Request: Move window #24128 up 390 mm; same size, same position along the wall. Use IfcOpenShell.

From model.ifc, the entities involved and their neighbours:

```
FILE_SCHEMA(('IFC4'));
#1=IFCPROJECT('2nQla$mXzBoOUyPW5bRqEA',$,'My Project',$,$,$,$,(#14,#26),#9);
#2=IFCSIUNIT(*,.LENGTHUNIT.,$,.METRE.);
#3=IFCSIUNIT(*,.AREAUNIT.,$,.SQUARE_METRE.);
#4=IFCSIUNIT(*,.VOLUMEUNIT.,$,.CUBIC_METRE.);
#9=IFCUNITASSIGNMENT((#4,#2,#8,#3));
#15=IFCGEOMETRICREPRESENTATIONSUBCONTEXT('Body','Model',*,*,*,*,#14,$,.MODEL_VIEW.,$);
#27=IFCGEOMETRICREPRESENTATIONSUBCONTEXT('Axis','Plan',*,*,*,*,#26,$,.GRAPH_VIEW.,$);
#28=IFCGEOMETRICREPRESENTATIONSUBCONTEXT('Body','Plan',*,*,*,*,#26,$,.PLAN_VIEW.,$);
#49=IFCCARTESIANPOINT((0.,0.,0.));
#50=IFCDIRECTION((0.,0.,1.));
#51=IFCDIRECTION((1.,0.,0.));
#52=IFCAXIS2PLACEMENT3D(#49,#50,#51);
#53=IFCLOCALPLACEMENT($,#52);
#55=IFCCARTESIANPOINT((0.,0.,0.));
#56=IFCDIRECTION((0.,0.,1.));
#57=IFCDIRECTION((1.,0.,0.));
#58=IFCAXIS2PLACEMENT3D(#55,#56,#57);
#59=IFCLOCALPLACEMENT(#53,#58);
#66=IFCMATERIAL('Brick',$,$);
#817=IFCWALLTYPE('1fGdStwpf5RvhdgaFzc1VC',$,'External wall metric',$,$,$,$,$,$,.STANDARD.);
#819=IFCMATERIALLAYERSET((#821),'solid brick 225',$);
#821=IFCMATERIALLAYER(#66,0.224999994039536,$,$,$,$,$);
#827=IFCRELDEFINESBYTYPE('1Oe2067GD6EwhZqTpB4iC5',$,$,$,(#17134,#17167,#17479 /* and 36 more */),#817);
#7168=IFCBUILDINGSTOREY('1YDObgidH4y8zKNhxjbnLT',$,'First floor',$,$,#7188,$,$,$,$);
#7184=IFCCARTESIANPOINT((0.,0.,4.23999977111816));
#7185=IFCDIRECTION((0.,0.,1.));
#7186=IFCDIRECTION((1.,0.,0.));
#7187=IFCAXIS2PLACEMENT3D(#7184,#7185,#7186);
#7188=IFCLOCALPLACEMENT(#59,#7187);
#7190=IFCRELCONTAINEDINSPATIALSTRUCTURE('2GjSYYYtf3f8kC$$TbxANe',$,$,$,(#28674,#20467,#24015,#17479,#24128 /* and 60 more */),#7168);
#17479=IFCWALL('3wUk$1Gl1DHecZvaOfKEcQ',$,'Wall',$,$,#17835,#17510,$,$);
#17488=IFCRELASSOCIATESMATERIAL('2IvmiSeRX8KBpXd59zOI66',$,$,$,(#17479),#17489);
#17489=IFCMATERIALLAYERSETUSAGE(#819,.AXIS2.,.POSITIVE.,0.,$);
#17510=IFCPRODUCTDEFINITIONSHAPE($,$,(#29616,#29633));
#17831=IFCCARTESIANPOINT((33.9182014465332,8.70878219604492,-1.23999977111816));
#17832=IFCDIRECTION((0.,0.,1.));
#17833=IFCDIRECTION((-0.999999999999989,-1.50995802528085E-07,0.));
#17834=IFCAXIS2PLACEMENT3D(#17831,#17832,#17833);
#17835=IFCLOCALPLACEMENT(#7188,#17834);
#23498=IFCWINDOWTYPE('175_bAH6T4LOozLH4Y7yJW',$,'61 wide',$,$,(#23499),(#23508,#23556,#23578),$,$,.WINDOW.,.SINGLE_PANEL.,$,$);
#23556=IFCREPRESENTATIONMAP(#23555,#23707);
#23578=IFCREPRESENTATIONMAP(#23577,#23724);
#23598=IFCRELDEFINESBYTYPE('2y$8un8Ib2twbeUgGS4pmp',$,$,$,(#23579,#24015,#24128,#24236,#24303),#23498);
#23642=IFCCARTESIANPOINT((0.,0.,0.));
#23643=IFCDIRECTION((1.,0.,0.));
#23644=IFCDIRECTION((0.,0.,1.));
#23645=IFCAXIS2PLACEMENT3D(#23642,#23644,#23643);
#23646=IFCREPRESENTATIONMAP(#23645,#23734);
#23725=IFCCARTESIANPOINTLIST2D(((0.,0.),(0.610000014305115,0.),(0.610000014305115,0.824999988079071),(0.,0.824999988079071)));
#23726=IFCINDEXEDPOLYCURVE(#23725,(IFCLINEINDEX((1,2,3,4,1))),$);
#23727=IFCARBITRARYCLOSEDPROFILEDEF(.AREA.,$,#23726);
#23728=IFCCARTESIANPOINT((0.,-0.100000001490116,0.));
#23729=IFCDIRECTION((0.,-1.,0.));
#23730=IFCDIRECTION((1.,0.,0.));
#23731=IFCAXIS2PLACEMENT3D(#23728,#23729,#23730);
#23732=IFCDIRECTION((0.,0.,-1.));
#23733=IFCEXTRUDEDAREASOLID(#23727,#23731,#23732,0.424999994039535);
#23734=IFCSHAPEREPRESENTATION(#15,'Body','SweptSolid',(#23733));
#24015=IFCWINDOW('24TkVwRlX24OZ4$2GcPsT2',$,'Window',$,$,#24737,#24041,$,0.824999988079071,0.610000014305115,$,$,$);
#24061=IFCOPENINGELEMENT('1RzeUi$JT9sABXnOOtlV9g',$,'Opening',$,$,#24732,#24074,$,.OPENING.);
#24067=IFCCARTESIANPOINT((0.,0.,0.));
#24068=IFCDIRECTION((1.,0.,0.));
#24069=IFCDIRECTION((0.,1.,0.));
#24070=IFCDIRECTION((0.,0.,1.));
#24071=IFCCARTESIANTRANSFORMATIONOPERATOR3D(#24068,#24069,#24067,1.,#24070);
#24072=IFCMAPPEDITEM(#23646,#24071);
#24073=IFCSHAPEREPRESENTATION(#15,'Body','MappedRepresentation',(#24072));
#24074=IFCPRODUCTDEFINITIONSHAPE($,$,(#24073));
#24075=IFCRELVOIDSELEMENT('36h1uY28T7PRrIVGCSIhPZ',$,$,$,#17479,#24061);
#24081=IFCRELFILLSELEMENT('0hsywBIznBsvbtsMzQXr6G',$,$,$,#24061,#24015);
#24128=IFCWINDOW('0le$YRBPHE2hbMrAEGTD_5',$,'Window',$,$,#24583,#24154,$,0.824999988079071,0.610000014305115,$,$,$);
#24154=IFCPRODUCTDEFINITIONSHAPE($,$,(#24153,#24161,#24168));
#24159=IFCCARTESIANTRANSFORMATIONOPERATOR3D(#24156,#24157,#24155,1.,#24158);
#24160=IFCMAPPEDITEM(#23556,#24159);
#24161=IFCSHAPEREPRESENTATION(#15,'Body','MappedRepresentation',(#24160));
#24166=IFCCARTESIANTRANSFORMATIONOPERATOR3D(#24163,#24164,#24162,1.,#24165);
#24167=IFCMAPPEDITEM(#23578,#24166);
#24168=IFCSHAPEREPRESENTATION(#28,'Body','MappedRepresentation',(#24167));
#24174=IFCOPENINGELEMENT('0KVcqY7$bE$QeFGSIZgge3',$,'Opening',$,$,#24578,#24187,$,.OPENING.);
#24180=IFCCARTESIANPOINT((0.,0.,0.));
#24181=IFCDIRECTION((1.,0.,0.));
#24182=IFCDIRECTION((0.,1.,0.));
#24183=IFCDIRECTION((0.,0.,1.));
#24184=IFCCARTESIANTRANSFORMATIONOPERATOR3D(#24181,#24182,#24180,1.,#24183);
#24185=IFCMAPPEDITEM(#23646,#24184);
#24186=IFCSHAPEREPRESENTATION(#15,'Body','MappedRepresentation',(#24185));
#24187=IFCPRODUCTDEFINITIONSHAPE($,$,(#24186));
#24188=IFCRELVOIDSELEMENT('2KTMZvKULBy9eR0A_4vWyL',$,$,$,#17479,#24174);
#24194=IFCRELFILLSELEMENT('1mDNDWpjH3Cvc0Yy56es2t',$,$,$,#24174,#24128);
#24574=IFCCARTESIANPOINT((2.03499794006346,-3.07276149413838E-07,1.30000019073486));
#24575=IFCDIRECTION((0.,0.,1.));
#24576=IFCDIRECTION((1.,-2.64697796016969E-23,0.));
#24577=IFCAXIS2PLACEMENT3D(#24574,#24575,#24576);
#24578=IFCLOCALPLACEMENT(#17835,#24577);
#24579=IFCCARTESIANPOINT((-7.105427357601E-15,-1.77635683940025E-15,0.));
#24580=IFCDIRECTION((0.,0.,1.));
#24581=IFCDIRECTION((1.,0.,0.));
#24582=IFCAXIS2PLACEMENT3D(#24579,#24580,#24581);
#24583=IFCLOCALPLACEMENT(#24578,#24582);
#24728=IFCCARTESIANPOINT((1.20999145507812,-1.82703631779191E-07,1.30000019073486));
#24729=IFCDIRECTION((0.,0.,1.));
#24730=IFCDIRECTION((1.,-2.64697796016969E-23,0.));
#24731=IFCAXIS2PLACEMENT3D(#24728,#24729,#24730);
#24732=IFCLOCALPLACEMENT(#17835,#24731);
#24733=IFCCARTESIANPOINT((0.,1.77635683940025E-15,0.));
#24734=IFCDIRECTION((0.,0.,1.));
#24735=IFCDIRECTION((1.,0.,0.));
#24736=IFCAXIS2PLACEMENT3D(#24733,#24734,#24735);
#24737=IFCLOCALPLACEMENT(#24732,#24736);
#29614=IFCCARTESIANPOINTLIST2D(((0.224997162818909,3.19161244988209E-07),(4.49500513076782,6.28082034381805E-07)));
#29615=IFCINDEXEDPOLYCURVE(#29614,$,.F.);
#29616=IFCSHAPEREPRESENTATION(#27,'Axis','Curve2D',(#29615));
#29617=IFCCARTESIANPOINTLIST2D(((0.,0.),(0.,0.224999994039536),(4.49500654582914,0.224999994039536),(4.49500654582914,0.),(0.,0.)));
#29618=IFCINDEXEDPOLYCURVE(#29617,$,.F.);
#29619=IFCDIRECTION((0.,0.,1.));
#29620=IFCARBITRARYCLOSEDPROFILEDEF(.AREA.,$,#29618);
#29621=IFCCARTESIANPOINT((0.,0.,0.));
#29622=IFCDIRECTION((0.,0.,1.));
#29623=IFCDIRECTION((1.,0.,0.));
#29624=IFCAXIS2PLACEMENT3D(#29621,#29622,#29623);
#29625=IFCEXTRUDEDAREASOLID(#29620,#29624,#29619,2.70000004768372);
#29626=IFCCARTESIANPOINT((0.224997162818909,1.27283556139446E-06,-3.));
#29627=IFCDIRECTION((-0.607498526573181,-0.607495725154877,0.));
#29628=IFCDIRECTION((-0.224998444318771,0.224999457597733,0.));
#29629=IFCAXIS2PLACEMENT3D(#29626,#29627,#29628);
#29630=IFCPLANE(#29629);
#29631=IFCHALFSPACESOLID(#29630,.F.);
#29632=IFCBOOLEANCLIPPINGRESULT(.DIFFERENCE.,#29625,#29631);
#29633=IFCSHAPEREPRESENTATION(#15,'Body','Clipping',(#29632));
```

```python
import numpy as np
import ifcopenshell
import ifcopenshell.api.geometry
import ifcopenshell.util.placement
import ifcopenshell.util.unit

model = ifcopenshell.open("model.ifc")
unit_scale = ifcopenshell.util.unit.calculate_unit_scale(model)

window = model.by_id(24128)
opening = window.FillsVoids[0].RelatingOpeningElement
dz = 0.39

shift = np.array([0.0, 0.0, dz])
# The window is placed relative to its opening, so it follows when the opening moves.
matrix = ifcopenshell.util.placement.get_local_placement(opening.ObjectPlacement)
matrix[:3, 3] += shift
ifcopenshell.api.geometry.edit_object_placement(
    model, product=opening, matrix=matrix, is_si=False, should_transform_children=True
)

print(f"moved by {dz * unit_scale:+.3f} m")

model.write("model_updated.ifc")
```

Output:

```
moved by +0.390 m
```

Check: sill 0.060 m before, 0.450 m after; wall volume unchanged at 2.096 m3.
